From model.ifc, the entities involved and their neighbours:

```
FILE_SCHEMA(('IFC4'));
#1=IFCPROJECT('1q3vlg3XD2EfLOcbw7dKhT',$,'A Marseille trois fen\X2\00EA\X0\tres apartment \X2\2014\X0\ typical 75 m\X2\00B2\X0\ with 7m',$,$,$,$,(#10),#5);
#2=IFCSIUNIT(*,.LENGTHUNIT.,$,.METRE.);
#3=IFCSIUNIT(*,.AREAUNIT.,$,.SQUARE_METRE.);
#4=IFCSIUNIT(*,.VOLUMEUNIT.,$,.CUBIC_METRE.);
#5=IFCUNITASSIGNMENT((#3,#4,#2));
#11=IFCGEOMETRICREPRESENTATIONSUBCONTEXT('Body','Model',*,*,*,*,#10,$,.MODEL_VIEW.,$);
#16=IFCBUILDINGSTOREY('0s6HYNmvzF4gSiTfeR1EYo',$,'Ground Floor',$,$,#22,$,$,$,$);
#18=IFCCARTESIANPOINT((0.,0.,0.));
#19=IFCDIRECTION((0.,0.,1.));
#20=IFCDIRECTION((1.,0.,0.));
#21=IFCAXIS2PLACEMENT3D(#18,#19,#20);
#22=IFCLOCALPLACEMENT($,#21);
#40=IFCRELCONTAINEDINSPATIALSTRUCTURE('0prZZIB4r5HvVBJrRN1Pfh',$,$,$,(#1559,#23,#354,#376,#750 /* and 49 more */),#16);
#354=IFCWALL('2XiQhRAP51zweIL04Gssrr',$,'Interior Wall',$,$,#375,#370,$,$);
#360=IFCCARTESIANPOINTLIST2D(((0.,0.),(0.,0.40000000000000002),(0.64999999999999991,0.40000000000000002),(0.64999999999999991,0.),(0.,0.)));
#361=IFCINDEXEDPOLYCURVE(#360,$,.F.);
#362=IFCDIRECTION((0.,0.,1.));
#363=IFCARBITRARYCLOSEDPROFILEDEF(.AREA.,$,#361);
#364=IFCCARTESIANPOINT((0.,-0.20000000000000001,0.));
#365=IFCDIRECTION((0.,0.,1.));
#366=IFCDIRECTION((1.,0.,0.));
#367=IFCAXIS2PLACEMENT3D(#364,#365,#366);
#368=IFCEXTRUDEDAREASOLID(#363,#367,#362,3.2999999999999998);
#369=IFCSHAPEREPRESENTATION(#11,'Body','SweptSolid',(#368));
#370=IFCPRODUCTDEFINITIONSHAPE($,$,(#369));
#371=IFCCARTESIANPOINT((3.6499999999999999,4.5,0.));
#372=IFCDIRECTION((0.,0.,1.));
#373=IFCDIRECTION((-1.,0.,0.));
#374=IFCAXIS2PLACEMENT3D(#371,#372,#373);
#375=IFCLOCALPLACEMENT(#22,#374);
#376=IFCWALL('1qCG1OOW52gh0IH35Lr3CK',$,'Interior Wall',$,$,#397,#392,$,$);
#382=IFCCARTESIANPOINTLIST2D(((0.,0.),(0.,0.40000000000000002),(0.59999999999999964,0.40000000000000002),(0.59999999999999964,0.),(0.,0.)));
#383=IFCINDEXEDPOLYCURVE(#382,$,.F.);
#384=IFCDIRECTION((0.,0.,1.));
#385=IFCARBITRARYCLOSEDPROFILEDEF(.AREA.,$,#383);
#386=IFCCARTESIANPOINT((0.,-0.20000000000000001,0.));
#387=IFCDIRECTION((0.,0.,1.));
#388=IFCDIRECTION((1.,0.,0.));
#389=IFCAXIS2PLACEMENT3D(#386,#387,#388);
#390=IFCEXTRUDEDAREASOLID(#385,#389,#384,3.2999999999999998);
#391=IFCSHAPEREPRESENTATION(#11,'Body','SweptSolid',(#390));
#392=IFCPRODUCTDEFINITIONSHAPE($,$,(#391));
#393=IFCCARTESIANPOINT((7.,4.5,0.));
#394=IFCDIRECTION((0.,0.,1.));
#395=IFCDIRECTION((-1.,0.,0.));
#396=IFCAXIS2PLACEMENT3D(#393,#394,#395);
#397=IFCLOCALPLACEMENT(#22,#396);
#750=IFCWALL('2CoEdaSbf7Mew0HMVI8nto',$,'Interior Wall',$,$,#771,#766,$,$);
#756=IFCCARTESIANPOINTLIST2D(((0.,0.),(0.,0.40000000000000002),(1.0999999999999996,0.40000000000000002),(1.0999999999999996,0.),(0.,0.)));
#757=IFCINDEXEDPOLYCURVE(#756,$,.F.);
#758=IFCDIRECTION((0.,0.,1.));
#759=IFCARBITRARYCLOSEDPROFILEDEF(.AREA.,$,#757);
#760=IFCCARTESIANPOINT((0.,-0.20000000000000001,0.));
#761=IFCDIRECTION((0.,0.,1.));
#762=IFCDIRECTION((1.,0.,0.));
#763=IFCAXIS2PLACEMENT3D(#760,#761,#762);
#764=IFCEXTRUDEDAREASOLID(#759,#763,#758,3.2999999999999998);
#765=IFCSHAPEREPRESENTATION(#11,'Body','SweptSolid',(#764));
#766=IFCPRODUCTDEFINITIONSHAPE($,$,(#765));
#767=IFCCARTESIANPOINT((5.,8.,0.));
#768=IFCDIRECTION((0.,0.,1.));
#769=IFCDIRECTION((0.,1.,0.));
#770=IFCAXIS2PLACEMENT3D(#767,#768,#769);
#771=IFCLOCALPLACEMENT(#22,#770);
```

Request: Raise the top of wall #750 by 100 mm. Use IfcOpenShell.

```python
import ifcopenshell
import ifcopenshell.geom
import ifcopenshell.util.representation
import ifcopenshell.util.shape
import ifcopenshell.util.unit

model = ifcopenshell.open("model.ifc")
unit_scale = ifcopenshell.util.unit.calculate_unit_scale(model)
settings = ifcopenshell.geom.settings()


def volume(element):
    """Net volume in cubic metres, openings subtracted."""
    shape = ifcopenshell.geom.create_shape(settings, element)
    return ifcopenshell.util.shape.get_volume(shape.geometry)


wall = model.by_guid("2CoEdaSbf7Mew0HMVI8nto")
before = volume(wall)

body = ifcopenshell.util.representation.get_representation(wall, "Model", "Body")
solid = body.Items[0]
old_height = solid.Depth
solid.Depth += 0.1 / unit_scale
after = volume(wall)

print(f"height {old_height:g} -> {solid.Depth:g}, volume {before:.3f} -> {after:.3f} m3")

model.write("model_edited.ifc")
```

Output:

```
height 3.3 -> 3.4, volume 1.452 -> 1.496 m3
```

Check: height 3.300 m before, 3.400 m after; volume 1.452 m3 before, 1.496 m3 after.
